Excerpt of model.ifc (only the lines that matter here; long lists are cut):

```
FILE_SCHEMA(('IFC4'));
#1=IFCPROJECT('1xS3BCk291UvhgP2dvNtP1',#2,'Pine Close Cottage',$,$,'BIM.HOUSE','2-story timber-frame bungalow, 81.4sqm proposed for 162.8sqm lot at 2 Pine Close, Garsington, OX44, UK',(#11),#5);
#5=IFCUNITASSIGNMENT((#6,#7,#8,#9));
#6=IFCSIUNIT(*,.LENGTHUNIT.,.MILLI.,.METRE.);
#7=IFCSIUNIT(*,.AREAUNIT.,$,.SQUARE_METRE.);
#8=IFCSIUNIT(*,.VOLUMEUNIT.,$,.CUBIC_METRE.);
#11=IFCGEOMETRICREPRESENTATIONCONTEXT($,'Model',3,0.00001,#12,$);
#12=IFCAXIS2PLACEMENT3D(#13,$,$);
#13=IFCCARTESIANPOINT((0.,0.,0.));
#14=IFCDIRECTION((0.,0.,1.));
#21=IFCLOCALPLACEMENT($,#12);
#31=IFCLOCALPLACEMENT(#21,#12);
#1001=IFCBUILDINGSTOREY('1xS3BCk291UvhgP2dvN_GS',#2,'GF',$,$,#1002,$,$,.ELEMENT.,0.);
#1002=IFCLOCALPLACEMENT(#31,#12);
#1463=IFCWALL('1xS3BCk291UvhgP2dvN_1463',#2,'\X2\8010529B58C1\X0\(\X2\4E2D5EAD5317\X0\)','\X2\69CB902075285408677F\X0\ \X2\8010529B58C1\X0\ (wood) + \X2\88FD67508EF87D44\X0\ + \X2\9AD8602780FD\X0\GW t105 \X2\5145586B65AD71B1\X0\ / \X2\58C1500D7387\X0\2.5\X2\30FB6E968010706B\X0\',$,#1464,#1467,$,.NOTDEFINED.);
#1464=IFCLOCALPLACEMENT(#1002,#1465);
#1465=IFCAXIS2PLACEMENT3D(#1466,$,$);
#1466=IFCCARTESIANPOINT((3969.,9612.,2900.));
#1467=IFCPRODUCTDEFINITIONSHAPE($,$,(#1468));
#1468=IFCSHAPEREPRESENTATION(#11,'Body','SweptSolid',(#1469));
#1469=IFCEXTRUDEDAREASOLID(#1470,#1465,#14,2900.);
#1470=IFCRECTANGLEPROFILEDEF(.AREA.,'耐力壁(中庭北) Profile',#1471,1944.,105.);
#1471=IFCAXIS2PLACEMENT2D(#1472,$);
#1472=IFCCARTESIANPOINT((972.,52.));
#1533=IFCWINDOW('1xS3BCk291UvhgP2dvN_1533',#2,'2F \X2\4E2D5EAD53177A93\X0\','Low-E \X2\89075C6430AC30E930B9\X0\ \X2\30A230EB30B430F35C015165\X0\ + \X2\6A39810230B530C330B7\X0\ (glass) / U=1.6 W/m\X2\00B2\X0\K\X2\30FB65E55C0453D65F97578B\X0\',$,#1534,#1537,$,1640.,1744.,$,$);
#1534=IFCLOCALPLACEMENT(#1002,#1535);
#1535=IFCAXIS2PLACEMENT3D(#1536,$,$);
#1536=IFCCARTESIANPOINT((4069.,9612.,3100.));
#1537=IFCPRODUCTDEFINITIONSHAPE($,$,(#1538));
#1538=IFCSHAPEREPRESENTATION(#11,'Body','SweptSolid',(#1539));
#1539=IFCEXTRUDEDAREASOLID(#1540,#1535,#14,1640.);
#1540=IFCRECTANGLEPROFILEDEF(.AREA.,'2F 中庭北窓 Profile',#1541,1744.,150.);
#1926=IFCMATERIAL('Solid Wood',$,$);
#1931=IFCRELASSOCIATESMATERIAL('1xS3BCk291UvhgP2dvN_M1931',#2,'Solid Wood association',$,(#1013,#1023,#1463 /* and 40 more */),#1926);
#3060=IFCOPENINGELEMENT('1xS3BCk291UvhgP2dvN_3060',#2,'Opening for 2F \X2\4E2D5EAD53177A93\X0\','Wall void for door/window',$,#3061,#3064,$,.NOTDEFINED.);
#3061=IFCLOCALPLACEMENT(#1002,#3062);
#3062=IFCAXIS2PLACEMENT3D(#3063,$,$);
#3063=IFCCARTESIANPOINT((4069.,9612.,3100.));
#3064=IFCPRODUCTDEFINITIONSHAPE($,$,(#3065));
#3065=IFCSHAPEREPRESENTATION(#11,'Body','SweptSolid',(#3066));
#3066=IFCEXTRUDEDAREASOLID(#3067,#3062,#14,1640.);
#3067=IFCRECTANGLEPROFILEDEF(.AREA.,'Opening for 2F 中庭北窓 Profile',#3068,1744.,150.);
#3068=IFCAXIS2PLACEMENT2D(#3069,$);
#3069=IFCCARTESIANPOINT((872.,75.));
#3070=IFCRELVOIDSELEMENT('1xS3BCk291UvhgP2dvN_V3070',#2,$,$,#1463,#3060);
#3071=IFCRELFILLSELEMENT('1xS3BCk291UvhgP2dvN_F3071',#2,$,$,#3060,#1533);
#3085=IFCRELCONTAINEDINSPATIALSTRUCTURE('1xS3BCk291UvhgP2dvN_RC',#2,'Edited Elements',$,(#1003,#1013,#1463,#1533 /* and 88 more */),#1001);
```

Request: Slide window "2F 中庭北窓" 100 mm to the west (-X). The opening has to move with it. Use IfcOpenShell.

```python
import ifcopenshell
import ifcopenshell.api.geometry
import ifcopenshell.util.placement
import ifcopenshell.util.unit

model = ifcopenshell.open("model.ifc")
unit_scale = ifcopenshell.util.unit.calculate_unit_scale(model)

window = model.by_guid("1xS3BCk291UvhgP2dvN_1533")
opening = window.FillsVoids[0].RelatingOpeningElement
wall = opening.VoidsElements[0].RelatingBuildingElement

wall_matrix = ifcopenshell.util.placement.get_local_placement(wall.ObjectPlacement)
shift = wall_matrix[:3, 0] * -0.1 / unit_scale
before = ifcopenshell.util.placement.get_local_placement(window.ObjectPlacement)[:3, 3].copy()

# The window is not placed relative to its opening, so move both.
for product in (opening, window):
    matrix = ifcopenshell.util.placement.get_local_placement(product.ObjectPlacement)
    matrix[:3, 3] += shift
    ifcopenshell.api.geometry.edit_object_placement(model, product=product, matrix=matrix, is_si=False)

after = ifcopenshell.util.placement.get_local_placement(window.ObjectPlacement)[:3, 3]
print("window moved by", (after - before).round(3) + 0.0)

model.write("model_v2.ifc")
```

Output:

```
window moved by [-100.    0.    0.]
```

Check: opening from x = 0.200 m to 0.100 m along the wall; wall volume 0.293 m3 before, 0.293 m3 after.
